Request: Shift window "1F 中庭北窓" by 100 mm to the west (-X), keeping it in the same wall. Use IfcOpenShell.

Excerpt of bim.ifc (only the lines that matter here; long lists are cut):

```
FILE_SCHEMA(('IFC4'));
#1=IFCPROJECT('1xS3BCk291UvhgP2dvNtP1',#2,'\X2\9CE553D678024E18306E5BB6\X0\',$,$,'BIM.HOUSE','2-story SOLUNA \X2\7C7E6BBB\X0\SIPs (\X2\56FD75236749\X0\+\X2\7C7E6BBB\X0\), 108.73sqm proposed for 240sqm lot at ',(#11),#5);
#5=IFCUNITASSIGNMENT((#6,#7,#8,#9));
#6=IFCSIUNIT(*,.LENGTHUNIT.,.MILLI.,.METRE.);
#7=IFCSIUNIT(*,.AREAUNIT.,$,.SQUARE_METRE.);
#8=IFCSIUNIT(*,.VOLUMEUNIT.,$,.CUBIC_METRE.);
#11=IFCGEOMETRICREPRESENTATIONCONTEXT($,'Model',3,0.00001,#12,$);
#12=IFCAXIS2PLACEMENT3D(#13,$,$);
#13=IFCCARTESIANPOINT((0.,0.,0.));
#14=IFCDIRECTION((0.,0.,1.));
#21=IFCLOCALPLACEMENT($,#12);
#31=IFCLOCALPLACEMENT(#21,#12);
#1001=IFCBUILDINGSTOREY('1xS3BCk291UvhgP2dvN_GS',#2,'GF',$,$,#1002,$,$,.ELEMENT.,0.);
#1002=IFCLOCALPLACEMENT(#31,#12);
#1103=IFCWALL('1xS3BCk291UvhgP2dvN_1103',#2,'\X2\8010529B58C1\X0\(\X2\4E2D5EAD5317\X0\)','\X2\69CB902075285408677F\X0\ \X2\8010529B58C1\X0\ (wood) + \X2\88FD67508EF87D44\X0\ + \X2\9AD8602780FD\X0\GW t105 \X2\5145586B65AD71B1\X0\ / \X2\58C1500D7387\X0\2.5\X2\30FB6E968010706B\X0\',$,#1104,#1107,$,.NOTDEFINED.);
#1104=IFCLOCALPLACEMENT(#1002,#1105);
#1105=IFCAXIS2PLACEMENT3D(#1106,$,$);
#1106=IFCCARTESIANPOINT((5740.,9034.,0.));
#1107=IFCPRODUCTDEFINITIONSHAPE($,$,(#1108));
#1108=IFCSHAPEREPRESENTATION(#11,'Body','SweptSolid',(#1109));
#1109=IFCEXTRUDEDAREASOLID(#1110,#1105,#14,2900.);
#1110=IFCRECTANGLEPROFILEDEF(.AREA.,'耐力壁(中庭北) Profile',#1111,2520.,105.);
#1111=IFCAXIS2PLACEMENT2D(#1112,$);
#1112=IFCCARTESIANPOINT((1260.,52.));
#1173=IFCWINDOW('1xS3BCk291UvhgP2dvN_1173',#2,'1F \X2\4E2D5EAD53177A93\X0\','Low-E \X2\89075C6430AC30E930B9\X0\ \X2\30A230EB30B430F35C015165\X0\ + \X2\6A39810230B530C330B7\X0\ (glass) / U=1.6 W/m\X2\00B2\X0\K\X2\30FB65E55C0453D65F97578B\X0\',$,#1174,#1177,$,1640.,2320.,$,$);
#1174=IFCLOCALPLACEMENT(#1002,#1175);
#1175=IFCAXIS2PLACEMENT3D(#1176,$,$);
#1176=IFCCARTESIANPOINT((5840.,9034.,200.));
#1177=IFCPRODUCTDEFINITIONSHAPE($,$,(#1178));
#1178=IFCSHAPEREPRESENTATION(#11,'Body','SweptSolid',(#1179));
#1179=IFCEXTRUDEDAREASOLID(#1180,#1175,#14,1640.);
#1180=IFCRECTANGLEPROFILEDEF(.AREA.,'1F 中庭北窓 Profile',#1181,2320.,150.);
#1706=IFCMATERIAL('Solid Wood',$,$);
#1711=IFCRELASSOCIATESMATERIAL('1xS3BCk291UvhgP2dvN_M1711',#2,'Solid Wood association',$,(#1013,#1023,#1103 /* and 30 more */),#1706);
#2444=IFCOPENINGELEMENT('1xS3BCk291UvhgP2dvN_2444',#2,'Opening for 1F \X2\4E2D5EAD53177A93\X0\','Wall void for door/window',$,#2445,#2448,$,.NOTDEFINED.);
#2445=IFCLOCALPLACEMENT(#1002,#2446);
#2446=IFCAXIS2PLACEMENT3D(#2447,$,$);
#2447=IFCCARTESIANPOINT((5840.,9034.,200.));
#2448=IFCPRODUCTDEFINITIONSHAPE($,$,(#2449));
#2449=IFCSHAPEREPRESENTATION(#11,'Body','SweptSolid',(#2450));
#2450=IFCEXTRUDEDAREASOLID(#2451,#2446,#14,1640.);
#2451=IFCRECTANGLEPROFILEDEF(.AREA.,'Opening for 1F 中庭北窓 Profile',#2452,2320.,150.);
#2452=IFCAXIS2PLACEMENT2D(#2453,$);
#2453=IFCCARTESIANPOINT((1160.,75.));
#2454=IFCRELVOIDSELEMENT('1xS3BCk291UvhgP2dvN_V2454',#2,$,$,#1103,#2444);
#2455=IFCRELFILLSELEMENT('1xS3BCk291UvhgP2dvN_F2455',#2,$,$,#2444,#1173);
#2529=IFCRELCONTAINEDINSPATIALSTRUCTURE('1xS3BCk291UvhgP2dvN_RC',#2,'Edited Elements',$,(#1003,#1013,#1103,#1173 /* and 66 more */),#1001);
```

```python
import ifcopenshell
import ifcopenshell.api.geometry
import ifcopenshell.util.placement
import ifcopenshell.util.unit

model = ifcopenshell.open("bim.ifc")
unit_scale = ifcopenshell.util.unit.calculate_unit_scale(model)

window = model.by_id(1173)
opening = window.FillsVoids[0].RelatingOpeningElement
wall = opening.VoidsElements[0].RelatingBuildingElement

wall_matrix = ifcopenshell.util.placement.get_local_placement(wall.ObjectPlacement)
shift = wall_matrix[:3, 0] * -0.1 / unit_scale
before = ifcopenshell.util.placement.get_local_placement(window.ObjectPlacement)[:3, 3].copy()

# The window is not placed relative to its opening, so move both.
for product in (opening, window):
    matrix = ifcopenshell.util.placement.get_local_placement(product.ObjectPlacement)
    matrix[:3, 3] += shift
    ifcopenshell.api.geometry.edit_object_placement(model, product=product, matrix=matrix, is_si=False)

after = ifcopenshell.util.placement.get_local_placement(window.ObjectPlacement)[:3, 3]
print("window moved by", (after - before).round(3) + 0.0)

model.write("bim_edited.ifc")
```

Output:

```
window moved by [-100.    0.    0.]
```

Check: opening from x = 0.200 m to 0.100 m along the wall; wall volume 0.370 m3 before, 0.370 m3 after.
